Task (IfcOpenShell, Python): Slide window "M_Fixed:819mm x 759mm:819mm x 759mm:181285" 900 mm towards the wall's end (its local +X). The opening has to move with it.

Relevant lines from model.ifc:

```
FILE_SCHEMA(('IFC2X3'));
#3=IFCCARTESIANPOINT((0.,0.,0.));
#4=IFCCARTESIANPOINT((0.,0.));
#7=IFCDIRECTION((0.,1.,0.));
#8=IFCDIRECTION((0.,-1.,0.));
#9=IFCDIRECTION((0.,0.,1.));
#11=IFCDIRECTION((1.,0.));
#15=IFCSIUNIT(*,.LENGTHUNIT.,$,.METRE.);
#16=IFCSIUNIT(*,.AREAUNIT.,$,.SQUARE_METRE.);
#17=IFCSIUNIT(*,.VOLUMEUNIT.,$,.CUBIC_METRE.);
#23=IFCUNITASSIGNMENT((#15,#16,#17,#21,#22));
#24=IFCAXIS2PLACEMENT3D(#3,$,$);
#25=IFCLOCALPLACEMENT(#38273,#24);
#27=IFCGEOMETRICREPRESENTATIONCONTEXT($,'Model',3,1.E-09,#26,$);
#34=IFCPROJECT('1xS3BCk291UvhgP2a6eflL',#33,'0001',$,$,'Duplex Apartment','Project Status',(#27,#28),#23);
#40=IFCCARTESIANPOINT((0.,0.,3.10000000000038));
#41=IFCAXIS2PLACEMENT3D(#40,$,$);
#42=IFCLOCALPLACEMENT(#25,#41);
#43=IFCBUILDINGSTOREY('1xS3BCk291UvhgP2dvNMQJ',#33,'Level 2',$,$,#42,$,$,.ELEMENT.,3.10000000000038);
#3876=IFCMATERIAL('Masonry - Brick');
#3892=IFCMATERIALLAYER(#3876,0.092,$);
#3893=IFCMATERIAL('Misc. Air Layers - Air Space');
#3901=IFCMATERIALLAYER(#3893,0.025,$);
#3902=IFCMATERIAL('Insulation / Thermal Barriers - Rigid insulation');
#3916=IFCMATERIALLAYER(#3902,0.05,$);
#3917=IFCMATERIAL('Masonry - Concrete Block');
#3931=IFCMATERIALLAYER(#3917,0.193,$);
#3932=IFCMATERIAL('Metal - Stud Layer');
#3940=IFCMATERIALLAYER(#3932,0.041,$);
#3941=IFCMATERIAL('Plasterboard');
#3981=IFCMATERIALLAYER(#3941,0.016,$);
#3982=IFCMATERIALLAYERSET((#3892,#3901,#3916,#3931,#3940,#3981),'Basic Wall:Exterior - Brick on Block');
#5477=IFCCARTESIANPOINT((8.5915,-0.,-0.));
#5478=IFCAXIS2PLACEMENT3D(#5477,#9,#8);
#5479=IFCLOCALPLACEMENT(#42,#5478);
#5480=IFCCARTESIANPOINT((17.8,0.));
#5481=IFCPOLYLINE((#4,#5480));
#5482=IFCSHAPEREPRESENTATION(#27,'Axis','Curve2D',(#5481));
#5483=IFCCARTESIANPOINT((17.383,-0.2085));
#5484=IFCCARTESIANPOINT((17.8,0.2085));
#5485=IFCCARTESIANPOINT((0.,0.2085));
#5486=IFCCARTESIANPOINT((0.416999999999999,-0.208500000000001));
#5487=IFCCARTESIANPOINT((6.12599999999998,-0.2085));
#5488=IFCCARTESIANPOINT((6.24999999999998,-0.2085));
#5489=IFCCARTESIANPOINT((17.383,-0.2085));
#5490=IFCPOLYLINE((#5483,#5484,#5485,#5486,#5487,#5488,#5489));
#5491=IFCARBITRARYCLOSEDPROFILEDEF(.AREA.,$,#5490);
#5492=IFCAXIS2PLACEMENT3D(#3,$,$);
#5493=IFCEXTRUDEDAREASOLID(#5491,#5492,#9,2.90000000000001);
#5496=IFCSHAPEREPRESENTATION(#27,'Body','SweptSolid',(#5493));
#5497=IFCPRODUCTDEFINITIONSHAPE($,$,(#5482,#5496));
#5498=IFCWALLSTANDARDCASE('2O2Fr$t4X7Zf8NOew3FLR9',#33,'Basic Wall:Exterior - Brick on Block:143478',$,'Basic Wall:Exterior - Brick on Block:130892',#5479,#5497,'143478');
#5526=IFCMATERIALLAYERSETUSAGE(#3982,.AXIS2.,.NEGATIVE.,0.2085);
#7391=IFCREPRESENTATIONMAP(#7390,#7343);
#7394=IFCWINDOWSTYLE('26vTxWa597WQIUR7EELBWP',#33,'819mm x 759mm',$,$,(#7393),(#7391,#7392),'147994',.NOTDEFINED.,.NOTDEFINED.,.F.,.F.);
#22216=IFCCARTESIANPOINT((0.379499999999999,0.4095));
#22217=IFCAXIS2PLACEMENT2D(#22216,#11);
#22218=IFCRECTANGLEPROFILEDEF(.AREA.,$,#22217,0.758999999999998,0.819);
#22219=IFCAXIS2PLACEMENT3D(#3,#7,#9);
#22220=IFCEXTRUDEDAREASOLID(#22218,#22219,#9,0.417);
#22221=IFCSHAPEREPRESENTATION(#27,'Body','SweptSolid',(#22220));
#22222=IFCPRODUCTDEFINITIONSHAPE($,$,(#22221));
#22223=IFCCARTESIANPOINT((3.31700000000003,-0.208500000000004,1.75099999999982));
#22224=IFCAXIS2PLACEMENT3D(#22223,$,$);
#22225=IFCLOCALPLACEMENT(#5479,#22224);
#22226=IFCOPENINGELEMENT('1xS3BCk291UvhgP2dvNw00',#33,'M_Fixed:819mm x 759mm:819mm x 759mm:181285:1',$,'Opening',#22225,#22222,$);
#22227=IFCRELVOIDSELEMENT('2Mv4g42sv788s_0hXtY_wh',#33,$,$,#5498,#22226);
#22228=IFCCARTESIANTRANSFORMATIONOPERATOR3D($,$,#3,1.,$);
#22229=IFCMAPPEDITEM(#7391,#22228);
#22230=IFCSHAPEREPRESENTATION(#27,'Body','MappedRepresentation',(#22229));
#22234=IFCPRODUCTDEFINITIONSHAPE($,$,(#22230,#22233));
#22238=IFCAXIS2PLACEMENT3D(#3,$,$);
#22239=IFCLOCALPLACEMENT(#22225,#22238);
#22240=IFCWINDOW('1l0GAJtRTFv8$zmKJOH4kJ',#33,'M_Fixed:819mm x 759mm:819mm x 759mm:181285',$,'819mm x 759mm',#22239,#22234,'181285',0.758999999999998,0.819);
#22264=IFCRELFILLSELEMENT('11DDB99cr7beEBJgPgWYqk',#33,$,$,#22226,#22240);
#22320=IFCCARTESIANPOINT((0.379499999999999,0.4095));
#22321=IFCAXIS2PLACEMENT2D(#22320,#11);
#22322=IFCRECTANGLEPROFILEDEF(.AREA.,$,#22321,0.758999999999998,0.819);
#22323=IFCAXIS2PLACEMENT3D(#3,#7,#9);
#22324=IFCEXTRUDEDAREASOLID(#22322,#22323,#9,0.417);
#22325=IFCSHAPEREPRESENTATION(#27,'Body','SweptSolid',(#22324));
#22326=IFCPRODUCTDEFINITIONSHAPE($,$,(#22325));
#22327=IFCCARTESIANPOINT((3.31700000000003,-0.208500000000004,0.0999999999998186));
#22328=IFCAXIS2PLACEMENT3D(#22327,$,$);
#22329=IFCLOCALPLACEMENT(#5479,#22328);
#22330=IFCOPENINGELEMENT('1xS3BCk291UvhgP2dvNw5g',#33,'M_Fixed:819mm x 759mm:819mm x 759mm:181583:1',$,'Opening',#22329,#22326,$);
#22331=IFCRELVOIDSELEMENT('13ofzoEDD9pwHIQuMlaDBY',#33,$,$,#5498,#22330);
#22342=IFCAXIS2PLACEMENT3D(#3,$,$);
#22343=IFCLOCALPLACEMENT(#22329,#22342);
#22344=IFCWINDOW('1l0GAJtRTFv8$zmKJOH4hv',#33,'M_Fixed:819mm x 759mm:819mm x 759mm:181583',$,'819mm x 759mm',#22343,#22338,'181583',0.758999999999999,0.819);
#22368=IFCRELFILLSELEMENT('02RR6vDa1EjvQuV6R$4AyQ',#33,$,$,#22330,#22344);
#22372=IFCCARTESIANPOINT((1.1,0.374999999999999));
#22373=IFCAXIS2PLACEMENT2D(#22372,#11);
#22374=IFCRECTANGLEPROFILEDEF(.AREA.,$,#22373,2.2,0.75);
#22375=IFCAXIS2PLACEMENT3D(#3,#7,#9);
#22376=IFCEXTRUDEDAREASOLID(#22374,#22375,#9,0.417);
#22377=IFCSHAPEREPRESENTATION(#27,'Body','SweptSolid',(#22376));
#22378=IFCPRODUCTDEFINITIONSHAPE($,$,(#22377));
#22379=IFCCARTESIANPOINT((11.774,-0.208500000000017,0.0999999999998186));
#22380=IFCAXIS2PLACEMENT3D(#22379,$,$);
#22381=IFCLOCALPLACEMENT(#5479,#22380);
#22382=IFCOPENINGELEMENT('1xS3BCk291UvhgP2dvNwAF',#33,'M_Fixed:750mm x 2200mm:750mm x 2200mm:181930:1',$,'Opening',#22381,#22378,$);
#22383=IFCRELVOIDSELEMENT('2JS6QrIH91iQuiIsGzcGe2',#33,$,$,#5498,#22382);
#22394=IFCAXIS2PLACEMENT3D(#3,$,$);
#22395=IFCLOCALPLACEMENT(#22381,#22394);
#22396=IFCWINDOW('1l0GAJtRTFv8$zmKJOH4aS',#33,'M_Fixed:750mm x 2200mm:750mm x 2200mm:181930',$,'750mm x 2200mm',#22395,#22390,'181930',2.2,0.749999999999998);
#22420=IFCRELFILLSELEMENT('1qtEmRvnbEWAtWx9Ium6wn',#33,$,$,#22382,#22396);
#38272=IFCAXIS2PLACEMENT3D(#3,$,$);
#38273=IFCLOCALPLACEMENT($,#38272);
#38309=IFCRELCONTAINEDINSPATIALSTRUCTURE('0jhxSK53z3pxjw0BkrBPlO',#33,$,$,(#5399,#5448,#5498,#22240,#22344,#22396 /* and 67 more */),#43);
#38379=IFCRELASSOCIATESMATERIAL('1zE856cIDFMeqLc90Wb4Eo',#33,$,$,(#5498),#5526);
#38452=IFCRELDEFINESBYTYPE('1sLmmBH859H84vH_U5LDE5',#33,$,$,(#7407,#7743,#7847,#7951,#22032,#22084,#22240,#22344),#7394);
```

```python
import ifcopenshell
import ifcopenshell.api.geometry
import ifcopenshell.util.placement

model = ifcopenshell.open("model.ifc")

window = model.by_guid("1l0GAJtRTFv8$zmKJOH4kJ")
opening = window.FillsVoids[0].RelatingOpeningElement
wall = opening.VoidsElements[0].RelatingBuildingElement

wall_matrix = ifcopenshell.util.placement.get_local_placement(wall.ObjectPlacement)
shift = wall_matrix[:3, 0] * 0.9
before = ifcopenshell.util.placement.get_local_placement(window.ObjectPlacement)[:3, 3].copy()

# The window is placed relative to its opening, so it follows when the opening moves.
matrix = ifcopenshell.util.placement.get_local_placement(opening.ObjectPlacement)
matrix[:3, 3] += shift
ifcopenshell.api.geometry.edit_object_placement(
    model, product=opening, matrix=matrix, is_si=False, should_transform_children=True
)

after = ifcopenshell.util.placement.get_local_placement(window.ObjectPlacement)[:3, 3]
print("window moved by", (after - before).round(3) + 0.0)

model.write("model-out.ifc")
```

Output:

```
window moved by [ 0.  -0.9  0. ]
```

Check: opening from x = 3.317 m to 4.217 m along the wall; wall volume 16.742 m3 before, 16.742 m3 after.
